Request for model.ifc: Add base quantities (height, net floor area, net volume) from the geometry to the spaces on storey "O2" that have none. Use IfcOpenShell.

First a look at what the model holds.

```python
import ifcopenshell
import ifcopenshell.util.element
import ifcopenshell.util.unit

model = ifcopenshell.open("model.ifc")
print(model.schema)
for unit_type in ("LENGTHUNIT", "AREAUNIT", "VOLUMEUNIT"):
    print(unit_type, ifcopenshell.util.unit.calculate_unit_scale(model, unit_type))
storey = next(s for s in model.by_type("IfcBuildingStorey") if s.Name == "O2")
spaces = [e for e in ifcopenshell.util.element.get_decomposition(storey) if e.is_a("IfcSpace")]
for e in sorted(spaces, key=lambda e: e.id()):
    print(e.id(), e.is_a(), e.Name, list(ifcopenshell.util.element.get_psets(e, qtos_only=True)), sep=" | ")
```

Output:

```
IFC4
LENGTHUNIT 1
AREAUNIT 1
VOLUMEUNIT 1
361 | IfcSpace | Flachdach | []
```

```python
import ifcopenshell
import ifcopenshell.api.pset
import ifcopenshell.geom
import ifcopenshell.util.element
import ifcopenshell.util.shape
import ifcopenshell.util.unit

model = ifcopenshell.open("model.ifc")
unit_scale = ifcopenshell.util.unit.calculate_unit_scale(model)
area_scale = ifcopenshell.util.unit.calculate_unit_scale(model, "AREAUNIT")
volume_scale = ifcopenshell.util.unit.calculate_unit_scale(model, "VOLUMEUNIT")
settings = ifcopenshell.geom.settings()

storey = next(s for s in model.by_type("IfcBuildingStorey") if s.Name == "O2")
spaces = [e for e in ifcopenshell.util.element.get_decomposition(storey) if e.is_a("IfcSpace")]

for e in sorted(spaces, key=lambda e: e.id()):
    if ifcopenshell.util.element.get_psets(e, qtos_only=True, should_inherit=False):
        continue
    # Geometry comes back in metres, in the element's own axes.
    shape = ifcopenshell.geom.create_shape(settings, e)
    values = {
        "Height": ifcopenshell.util.shape.get_z(shape.geometry) / unit_scale,
        "NetFloorArea": ifcopenshell.util.shape.get_footprint_area(shape.geometry) / area_scale,
        "NetVolume": ifcopenshell.util.shape.get_volume(shape.geometry) / volume_scale,
    }
    qto = ifcopenshell.api.pset.add_qto(model, product=e, name="Qto_SpaceBaseQuantities")
    ifcopenshell.api.pset.edit_qto(model, qto=qto, properties=values)
    print(e.id(), {k: round(v, 3) for k, v in values.items()})

model.write("model_edited.ifc")
```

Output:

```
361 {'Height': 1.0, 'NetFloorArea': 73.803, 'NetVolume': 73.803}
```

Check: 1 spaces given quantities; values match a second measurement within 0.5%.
